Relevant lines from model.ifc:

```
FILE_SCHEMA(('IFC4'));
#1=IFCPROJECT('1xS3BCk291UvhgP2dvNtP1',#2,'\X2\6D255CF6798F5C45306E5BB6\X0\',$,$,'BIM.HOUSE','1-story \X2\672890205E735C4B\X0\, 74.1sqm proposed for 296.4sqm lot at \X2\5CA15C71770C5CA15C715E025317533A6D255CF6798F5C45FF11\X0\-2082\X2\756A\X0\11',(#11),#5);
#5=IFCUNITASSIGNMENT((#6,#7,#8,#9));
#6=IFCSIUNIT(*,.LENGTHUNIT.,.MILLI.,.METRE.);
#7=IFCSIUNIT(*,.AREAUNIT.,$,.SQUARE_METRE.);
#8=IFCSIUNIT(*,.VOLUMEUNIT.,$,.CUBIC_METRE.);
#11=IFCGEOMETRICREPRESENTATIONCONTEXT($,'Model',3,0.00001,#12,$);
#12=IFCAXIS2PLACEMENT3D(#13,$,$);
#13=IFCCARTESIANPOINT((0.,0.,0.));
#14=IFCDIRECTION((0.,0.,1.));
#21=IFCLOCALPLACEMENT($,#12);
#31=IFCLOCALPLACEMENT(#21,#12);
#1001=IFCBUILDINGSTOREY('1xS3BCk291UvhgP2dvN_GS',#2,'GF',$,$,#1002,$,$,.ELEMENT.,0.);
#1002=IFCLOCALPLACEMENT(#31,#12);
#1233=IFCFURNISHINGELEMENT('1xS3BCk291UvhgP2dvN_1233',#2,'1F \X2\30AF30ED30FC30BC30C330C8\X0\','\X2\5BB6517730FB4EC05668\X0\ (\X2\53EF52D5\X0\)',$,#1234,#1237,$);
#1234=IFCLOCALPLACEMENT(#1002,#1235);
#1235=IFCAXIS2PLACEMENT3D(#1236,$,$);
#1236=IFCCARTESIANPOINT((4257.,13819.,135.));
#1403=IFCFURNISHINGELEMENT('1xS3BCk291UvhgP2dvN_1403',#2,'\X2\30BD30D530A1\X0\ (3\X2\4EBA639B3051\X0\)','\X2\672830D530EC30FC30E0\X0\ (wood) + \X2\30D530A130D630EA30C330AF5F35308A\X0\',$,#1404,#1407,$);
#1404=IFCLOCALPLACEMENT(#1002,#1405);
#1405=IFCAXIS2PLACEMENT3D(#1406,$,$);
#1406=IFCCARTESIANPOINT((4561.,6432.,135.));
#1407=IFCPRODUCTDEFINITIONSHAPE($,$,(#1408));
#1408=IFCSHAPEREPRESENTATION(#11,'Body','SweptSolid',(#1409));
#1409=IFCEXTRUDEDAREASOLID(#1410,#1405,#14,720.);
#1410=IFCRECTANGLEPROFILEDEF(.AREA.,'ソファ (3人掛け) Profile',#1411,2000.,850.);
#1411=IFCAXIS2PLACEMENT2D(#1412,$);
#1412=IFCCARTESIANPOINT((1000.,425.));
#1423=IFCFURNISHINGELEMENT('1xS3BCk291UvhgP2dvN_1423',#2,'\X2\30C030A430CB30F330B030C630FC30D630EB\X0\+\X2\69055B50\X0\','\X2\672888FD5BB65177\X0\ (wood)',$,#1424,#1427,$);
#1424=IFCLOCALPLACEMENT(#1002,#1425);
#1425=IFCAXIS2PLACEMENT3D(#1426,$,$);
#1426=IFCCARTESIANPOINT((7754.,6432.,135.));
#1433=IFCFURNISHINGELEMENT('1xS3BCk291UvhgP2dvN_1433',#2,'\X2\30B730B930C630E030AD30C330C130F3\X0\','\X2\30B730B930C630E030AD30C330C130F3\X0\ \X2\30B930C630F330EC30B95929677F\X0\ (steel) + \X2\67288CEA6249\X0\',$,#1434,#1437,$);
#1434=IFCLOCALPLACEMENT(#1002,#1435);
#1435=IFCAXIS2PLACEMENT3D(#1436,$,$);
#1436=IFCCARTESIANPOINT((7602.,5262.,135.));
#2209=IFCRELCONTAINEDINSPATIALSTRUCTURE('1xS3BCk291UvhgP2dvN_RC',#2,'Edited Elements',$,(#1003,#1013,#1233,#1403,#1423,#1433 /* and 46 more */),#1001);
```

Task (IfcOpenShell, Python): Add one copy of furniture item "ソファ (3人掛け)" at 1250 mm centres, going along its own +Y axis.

```python
import ifcopenshell
import ifcopenshell.api.geometry
import ifcopenshell.api.root
import ifcopenshell.util.element
import ifcopenshell.util.placement
import ifcopenshell.util.unit

model = ifcopenshell.open("model.ifc")
unit_scale = ifcopenshell.util.unit.calculate_unit_scale(model)


def reuse_history(source, copy):
    """copy_class also copies each property set's owner history, people and application; keep the originals."""
    for rel in copy.IsDefinedBy:
        if rel.is_a("IfcRelDefinesByProperties") and (history := rel.RelatingPropertyDefinition.OwnerHistory):
            rel.RelatingPropertyDefinition.OwnerHistory = source.OwnerHistory
            ifcopenshell.util.element.remove_deep2(model, history)


source = model.by_id(1403)
base = ifcopenshell.util.placement.get_local_placement(source.ObjectPlacement)
step = base[:3, 1] * 1.25 / unit_scale

for i in range(1, 2):
    copy = ifcopenshell.api.root.copy_class(model, product=source)
    copy.Representation = ifcopenshell.util.element.copy_deep(
        model, source.Representation, exclude=["IfcGeometricRepresentationContext", "IfcRepresentationMap"]
    )
    reuse_history(source, copy)
    matrix = base.copy()
    matrix[:3, 3] += i * step
    print("added at", matrix[:3, 3].round(3) + 0.0)
    ifcopenshell.api.geometry.edit_object_placement(model, product=copy, matrix=matrix, is_si=False)

model.write("model_edited.ifc")
```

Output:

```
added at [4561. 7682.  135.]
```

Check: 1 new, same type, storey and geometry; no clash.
